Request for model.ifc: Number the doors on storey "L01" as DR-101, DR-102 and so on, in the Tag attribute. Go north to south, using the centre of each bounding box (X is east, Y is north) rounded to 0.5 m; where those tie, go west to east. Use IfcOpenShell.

First a look at what the model holds.

```python
import ifcopenshell
import ifcopenshell.util.element
import ifcopenshell.util.placement

model = ifcopenshell.open("model.ifc")
print(model.schema)
storey = next(s for s in model.by_type("IfcBuildingStorey") if s.Name == "L01")
doors = [e for e in ifcopenshell.util.element.get_decomposition(storey) if e.is_a("IfcDoor")]
for e in sorted(doors, key=lambda e: e.id()):
    origin = ifcopenshell.util.placement.get_local_placement(e.ObjectPlacement)[:3, 3]
    print(e.id(), e.Tag, e.Name, origin.round(2) + 0.0, sep=" | ")
```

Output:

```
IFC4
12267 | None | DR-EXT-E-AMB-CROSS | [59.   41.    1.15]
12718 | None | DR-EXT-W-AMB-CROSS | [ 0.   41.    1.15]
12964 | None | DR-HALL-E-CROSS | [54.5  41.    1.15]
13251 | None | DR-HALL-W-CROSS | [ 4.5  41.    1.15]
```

```python
import ifcopenshell
import ifcopenshell.geom
import ifcopenshell.util.element
import ifcopenshell.util.shape

model = ifcopenshell.open("model.ifc")
settings = ifcopenshell.geom.settings()
settings.set("use-world-coords", True)


def centre(element):
    shape = ifcopenshell.geom.create_shape(settings, element)
    return ifcopenshell.util.shape.get_bbox_centroid(shape.geometry)


storey = next(s for s in model.by_type("IfcBuildingStorey") if s.Name == "L01")
doors = [e for e in ifcopenshell.util.element.get_decomposition(storey) if e.is_a("IfcDoor")]

# Insertion points can sit at a corner or the storey origin, so sort by the geometry (in metres).
centres = {e: centre(e) for e in doors}
doors.sort(key=lambda e: (-round(centres[e][1] / 0.5), centres[e][0]))

for i, e in enumerate(doors, start=1):
    number = f"DR-1{i:02d}"
    e.Tag = number
    print(e.id(), number)

model.write("model_updated.ifc")
```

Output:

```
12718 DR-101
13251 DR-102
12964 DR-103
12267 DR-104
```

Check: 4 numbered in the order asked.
